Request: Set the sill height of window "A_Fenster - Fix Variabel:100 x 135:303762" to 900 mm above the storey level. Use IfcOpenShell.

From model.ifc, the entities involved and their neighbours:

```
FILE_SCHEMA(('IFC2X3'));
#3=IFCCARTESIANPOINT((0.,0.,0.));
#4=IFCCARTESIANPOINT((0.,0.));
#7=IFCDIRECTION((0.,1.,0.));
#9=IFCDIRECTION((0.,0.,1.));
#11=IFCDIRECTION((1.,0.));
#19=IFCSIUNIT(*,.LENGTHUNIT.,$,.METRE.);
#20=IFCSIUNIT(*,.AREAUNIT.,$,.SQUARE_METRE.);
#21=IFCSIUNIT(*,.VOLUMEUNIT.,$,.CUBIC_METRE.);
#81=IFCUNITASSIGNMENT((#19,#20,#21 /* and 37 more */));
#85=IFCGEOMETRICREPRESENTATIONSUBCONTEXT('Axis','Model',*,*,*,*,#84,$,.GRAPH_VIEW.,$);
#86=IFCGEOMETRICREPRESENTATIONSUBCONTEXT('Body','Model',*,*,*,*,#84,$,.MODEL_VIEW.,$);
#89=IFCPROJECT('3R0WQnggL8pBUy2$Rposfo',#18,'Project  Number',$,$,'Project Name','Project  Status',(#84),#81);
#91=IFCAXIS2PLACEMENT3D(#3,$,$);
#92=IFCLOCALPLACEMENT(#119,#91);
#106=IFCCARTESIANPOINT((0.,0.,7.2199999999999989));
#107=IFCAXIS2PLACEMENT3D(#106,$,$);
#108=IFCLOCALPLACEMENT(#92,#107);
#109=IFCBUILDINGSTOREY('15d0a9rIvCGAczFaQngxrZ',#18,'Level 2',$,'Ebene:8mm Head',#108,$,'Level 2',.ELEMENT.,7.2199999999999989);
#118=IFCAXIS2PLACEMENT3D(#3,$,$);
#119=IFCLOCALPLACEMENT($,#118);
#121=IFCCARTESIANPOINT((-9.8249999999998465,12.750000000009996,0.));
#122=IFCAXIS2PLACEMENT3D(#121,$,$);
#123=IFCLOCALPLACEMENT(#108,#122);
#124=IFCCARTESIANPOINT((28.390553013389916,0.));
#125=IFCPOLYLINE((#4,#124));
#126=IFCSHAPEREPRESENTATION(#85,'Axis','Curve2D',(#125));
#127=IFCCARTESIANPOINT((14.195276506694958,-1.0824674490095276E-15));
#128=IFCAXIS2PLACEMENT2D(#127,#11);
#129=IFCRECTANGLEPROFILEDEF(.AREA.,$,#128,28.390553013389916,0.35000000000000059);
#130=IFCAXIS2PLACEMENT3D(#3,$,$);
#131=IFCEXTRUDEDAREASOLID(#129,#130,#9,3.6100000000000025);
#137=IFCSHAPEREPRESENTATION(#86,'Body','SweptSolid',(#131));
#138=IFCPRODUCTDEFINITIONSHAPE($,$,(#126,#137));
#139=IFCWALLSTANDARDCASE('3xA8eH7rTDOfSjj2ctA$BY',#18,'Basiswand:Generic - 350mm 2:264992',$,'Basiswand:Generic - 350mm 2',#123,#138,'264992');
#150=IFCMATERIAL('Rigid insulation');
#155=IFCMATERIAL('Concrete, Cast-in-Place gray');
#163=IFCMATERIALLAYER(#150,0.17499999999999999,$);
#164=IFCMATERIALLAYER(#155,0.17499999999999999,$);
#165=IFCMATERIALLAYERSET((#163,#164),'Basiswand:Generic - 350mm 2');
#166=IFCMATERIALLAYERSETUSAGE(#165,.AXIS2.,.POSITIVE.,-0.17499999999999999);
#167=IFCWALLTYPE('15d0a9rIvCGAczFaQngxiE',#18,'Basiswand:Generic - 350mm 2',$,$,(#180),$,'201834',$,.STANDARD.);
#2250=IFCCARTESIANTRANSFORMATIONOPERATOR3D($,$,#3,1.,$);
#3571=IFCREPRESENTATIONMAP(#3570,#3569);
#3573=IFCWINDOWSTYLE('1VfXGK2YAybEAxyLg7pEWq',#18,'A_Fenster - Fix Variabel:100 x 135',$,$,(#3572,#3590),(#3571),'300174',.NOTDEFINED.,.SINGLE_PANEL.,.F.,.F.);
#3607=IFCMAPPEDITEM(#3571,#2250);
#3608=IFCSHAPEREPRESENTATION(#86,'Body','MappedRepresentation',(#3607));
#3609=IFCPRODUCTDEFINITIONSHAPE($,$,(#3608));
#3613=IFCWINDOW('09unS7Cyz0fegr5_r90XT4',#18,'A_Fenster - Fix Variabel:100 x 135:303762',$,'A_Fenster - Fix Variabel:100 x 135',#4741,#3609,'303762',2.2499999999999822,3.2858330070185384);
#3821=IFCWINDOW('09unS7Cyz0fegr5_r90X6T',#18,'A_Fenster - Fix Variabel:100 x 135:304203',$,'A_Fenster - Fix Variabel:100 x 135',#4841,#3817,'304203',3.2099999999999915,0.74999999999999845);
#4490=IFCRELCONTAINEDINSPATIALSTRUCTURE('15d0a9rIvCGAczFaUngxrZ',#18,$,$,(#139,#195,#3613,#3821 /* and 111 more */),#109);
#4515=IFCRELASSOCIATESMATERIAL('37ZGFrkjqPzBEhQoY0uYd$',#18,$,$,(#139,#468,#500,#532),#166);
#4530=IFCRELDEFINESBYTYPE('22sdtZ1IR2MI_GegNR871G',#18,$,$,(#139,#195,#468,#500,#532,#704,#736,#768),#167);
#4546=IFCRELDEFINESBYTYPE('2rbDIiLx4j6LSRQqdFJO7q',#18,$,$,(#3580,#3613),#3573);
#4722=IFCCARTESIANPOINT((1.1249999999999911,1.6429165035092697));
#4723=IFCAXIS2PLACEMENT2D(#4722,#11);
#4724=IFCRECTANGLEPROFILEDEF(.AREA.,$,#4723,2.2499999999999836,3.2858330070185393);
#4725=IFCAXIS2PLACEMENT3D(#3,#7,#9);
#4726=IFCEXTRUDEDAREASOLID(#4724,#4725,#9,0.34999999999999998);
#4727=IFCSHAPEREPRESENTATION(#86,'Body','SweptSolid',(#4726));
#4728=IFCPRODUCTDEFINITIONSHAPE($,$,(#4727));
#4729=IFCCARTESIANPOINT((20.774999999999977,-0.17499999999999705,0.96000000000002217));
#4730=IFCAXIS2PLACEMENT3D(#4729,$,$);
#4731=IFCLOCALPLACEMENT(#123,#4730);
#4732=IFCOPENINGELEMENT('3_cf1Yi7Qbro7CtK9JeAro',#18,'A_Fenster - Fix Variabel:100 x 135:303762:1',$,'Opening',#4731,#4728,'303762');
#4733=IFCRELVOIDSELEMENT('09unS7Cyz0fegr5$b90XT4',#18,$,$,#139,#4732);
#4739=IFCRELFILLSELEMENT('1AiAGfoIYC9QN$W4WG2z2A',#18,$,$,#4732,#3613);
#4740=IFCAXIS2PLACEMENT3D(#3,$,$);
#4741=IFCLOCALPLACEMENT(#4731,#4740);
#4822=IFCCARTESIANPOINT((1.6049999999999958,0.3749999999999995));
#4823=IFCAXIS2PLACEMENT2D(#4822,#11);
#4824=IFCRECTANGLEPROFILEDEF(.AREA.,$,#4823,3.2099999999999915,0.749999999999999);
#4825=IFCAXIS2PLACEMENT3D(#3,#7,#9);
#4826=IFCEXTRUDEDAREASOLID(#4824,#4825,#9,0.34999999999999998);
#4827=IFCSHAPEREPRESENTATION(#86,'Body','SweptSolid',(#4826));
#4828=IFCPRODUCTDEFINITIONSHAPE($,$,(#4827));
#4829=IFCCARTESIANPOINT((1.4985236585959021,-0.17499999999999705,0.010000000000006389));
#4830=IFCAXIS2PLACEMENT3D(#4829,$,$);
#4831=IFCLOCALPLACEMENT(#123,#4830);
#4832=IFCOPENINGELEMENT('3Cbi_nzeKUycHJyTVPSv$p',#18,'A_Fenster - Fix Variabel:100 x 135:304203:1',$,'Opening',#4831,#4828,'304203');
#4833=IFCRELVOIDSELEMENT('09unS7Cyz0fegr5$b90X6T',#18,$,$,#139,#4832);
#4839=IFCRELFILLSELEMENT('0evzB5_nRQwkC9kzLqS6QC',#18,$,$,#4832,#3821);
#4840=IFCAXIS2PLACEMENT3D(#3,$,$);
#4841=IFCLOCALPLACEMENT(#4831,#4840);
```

```python
import numpy as np
import ifcopenshell
import ifcopenshell.api.geometry
import ifcopenshell.geom
import ifcopenshell.util.element
import ifcopenshell.util.placement
import ifcopenshell.util.shape
import ifcopenshell.util.unit

model = ifcopenshell.open("model.ifc")
unit_scale = ifcopenshell.util.unit.calculate_unit_scale(model)

window = model.by_guid("09unS7Cyz0fegr5_r90XT4")
opening = window.FillsVoids[0].RelatingOpeningElement
storey = ifcopenshell.util.element.get_container(window, ifc_class="IfcBuildingStorey")
level = ifcopenshell.util.placement.get_local_placement(storey.ObjectPlacement)[2, 3]

# The opening's origin need not be at the sill, so measure its lowest point.
shape = ifcopenshell.geom.create_shape(ifcopenshell.geom.settings(), opening)
bottom = ifcopenshell.util.shape.get_shape_bottom_elevation(shape, shape.geometry) / unit_scale
dz = level + 0.9 - bottom

shift = np.array([0.0, 0.0, dz])
# The window is placed relative to its opening, so it follows when the opening moves.
matrix = ifcopenshell.util.placement.get_local_placement(opening.ObjectPlacement)
matrix[:3, 3] += shift
ifcopenshell.api.geometry.edit_object_placement(
    model, product=opening, matrix=matrix, is_si=False, should_transform_children=True
)

print(f"moved by {dz * unit_scale:+.3f} m")

model.write("model_edited.ifc")
```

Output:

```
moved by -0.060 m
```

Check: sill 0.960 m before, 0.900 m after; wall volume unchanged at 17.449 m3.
